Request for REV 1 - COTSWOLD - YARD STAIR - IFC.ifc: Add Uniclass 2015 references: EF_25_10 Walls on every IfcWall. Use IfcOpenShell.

First a look at what the model holds.

```python
import ifcopenshell

model = ifcopenshell.open("REV 1 - COTSWOLD - YARD STAIR - IFC.ifc")
print(model.schema)
print("classifications:", [c.Name for c in model.by_type("IfcClassification")])
for ifc_class in ("IfcDoor", "IfcRoof", "IfcStair", "IfcWall", "IfcWindow"):
    print(ifc_class, len(model.by_type(ifc_class)))
```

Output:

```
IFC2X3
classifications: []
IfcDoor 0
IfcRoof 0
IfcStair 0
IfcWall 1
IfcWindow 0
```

```python
import ifcopenshell
import ifcopenshell.api.classification

model = ifcopenshell.open("REV 1 - COTSWOLD - YARD STAIR - IFC.ifc")

# IFC2X3 requires Source and Edition and has no link from the project to the system.
system = model.create_entity("IfcClassification", Source="NBS", Edition="2015", Name="Uniclass 2015")

codes = {
    "IfcWall": ("EF_25_10", "Walls"),
}
for ifc_class, (code, name) in codes.items():
    products = model.by_type(ifc_class)
    ifcopenshell.api.classification.add_reference(
        model, products=products, classification=system, identification=code, name=name
    )
    print(code, len(products))

model.write("REV 1 - COTSWOLD - YARD STAIR - IFC_updated.ifc")
```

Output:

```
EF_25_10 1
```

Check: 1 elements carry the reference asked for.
